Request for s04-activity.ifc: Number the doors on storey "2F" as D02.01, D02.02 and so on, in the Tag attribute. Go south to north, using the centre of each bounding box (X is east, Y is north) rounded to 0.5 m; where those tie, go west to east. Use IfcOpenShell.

First a look at what the model holds.

```python
import ifcopenshell
import ifcopenshell.util.element
import ifcopenshell.util.placement

model = ifcopenshell.open("s04-activity.ifc")
print(model.schema)
storey = next(s for s in model.by_type("IfcBuildingStorey") if s.Name == "2F")
doors = [e for e in ifcopenshell.util.element.get_decomposition(storey) if e.is_a("IfcDoor")]
for e in sorted(doors, key=lambda e: e.id()):
    origin = ifcopenshell.util.placement.get_local_placement(e.ObjectPlacement)[:3, 3]
    print(e.id(), e.Tag, e.Name, origin.round(2) + 0.0, sep=" | ")
```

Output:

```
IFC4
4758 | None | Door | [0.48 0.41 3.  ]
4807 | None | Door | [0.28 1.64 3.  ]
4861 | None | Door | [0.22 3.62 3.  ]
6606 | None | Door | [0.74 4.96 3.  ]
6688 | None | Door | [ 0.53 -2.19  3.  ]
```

```python
import ifcopenshell
import ifcopenshell.geom
import ifcopenshell.util.element
import ifcopenshell.util.shape

model = ifcopenshell.open("s04-activity.ifc")
settings = ifcopenshell.geom.settings()
settings.set("use-world-coords", True)


def centre(element):
    shape = ifcopenshell.geom.create_shape(settings, element)
    return ifcopenshell.util.shape.get_bbox_centroid(shape.geometry)


storey = next(s for s in model.by_type("IfcBuildingStorey") if s.Name == "2F")
doors = [e for e in ifcopenshell.util.element.get_decomposition(storey) if e.is_a("IfcDoor")]

# Insertion points can sit at a corner or the storey origin, so sort by the geometry (in metres).
centres = {e: centre(e) for e in doors}
doors.sort(key=lambda e: (round(centres[e][1] / 0.5), centres[e][0]))

for i, e in enumerate(doors, start=1):
    number = f"D02.{i:02d}"
    e.Tag = number
    print(e.id(), number)

model.write("s04-activity_updated.ifc")
```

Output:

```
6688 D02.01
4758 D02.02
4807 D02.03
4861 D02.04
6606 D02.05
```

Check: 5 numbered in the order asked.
